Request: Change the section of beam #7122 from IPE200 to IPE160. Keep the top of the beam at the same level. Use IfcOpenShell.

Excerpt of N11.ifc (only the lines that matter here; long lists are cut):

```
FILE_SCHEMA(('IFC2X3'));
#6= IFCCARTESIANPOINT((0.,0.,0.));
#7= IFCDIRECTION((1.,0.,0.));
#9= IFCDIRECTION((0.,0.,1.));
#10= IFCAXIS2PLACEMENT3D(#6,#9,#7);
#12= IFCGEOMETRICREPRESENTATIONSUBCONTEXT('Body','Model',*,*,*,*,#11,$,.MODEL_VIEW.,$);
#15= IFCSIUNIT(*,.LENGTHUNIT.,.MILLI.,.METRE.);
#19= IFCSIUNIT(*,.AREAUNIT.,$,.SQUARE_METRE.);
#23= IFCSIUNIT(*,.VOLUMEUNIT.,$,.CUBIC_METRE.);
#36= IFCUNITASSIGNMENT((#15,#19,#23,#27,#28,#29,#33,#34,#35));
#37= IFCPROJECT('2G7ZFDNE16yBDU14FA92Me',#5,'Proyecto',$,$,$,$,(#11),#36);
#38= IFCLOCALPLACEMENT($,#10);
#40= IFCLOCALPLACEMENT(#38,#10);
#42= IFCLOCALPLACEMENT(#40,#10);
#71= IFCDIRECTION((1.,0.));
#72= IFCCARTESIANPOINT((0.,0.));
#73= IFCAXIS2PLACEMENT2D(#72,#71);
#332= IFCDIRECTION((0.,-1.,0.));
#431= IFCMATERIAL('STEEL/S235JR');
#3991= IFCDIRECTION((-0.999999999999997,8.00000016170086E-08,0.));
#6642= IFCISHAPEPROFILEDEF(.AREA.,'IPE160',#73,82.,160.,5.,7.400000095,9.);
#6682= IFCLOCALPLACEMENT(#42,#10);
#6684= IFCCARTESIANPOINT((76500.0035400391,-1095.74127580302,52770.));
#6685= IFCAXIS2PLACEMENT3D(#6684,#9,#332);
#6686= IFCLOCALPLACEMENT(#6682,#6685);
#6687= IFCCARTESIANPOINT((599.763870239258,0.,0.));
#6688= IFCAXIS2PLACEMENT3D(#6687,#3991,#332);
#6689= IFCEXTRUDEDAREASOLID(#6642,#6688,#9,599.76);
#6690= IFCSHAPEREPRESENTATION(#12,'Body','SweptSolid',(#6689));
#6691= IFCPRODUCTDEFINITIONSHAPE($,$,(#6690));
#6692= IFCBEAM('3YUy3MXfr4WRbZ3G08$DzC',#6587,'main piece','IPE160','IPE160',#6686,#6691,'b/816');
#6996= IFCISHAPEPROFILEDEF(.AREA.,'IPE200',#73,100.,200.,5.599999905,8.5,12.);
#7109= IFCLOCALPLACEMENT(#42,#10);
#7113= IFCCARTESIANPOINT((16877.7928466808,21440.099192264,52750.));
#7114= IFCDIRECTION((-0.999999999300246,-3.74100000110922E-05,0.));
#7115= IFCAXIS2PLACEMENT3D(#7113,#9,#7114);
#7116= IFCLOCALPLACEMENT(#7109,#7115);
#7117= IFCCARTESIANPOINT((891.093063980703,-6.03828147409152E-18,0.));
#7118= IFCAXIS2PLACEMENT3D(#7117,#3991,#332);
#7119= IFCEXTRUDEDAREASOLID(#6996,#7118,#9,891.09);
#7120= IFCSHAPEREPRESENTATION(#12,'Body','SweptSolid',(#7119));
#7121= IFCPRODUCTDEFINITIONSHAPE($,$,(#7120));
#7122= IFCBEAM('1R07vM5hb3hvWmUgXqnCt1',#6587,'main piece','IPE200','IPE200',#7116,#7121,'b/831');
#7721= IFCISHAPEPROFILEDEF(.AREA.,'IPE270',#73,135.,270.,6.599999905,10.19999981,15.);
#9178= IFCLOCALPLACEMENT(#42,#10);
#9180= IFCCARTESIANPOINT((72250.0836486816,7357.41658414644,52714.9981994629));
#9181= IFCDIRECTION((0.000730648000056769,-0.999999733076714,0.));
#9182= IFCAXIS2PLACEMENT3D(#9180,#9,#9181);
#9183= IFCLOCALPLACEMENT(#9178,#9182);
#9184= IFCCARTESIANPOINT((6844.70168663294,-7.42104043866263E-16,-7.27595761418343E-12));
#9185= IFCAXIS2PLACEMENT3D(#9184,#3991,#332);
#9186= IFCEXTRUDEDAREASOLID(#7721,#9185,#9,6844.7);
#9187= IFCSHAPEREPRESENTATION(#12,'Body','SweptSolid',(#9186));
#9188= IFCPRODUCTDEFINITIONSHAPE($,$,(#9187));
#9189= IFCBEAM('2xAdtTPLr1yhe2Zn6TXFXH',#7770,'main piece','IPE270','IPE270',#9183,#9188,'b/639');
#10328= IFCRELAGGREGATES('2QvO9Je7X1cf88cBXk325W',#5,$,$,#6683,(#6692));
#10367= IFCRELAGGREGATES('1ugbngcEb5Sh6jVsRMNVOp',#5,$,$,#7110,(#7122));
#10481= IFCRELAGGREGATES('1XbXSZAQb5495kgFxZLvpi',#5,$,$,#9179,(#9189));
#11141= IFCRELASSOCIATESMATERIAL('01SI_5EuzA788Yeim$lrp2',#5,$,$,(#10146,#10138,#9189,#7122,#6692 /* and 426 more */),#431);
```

```python
import ifcopenshell
import ifcopenshell.util.element
import ifcopenshell.util.representation

model = ifcopenshell.open("N11.ifc")

member = model.by_guid("1R07vM5hb3hvWmUgXqnCt1")
source = next(p for p in model.by_type("IfcIShapeProfileDef") if p.ProfileName == "IPE160")

body = ifcopenshell.util.representation.get_representation(member, "Model", "Body")
solid = body.Items[0]
old_profile = solid.SweptArea

# Copy the section's sizes but keep this member's own profile position.
profile = ifcopenshell.util.element.copy(model, source)
# Profiles are centred, so shift by half the change in depth to hold the top.
shift = (old_profile.OverallDepth - profile.OverallDepth) / 2
x, y = old_profile.Position.Location.Coordinates
up = (0.0, 1.0)  # upwards, in the solid's own plane
location = model.createIfcCartesianPoint((x + up[0] * shift, y + up[1] * shift))
profile.Position = model.createIfcAxis2Placement2D(location, old_profile.Position.RefDirection)
solid.SweptArea = profile
if not model.get_total_inverses(old_profile):
    ifcopenshell.util.element.remove_deep2(model, old_profile)
member.Description = member.Description.replace("IPE200", "IPE160")
member.ObjectType = member.ObjectType.replace("IPE200", "IPE160")

print(solid.SweptArea)

model.write("N11_rev.ifc")
```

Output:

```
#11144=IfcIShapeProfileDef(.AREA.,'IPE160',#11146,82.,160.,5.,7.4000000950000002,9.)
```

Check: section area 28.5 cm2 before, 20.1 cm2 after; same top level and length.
